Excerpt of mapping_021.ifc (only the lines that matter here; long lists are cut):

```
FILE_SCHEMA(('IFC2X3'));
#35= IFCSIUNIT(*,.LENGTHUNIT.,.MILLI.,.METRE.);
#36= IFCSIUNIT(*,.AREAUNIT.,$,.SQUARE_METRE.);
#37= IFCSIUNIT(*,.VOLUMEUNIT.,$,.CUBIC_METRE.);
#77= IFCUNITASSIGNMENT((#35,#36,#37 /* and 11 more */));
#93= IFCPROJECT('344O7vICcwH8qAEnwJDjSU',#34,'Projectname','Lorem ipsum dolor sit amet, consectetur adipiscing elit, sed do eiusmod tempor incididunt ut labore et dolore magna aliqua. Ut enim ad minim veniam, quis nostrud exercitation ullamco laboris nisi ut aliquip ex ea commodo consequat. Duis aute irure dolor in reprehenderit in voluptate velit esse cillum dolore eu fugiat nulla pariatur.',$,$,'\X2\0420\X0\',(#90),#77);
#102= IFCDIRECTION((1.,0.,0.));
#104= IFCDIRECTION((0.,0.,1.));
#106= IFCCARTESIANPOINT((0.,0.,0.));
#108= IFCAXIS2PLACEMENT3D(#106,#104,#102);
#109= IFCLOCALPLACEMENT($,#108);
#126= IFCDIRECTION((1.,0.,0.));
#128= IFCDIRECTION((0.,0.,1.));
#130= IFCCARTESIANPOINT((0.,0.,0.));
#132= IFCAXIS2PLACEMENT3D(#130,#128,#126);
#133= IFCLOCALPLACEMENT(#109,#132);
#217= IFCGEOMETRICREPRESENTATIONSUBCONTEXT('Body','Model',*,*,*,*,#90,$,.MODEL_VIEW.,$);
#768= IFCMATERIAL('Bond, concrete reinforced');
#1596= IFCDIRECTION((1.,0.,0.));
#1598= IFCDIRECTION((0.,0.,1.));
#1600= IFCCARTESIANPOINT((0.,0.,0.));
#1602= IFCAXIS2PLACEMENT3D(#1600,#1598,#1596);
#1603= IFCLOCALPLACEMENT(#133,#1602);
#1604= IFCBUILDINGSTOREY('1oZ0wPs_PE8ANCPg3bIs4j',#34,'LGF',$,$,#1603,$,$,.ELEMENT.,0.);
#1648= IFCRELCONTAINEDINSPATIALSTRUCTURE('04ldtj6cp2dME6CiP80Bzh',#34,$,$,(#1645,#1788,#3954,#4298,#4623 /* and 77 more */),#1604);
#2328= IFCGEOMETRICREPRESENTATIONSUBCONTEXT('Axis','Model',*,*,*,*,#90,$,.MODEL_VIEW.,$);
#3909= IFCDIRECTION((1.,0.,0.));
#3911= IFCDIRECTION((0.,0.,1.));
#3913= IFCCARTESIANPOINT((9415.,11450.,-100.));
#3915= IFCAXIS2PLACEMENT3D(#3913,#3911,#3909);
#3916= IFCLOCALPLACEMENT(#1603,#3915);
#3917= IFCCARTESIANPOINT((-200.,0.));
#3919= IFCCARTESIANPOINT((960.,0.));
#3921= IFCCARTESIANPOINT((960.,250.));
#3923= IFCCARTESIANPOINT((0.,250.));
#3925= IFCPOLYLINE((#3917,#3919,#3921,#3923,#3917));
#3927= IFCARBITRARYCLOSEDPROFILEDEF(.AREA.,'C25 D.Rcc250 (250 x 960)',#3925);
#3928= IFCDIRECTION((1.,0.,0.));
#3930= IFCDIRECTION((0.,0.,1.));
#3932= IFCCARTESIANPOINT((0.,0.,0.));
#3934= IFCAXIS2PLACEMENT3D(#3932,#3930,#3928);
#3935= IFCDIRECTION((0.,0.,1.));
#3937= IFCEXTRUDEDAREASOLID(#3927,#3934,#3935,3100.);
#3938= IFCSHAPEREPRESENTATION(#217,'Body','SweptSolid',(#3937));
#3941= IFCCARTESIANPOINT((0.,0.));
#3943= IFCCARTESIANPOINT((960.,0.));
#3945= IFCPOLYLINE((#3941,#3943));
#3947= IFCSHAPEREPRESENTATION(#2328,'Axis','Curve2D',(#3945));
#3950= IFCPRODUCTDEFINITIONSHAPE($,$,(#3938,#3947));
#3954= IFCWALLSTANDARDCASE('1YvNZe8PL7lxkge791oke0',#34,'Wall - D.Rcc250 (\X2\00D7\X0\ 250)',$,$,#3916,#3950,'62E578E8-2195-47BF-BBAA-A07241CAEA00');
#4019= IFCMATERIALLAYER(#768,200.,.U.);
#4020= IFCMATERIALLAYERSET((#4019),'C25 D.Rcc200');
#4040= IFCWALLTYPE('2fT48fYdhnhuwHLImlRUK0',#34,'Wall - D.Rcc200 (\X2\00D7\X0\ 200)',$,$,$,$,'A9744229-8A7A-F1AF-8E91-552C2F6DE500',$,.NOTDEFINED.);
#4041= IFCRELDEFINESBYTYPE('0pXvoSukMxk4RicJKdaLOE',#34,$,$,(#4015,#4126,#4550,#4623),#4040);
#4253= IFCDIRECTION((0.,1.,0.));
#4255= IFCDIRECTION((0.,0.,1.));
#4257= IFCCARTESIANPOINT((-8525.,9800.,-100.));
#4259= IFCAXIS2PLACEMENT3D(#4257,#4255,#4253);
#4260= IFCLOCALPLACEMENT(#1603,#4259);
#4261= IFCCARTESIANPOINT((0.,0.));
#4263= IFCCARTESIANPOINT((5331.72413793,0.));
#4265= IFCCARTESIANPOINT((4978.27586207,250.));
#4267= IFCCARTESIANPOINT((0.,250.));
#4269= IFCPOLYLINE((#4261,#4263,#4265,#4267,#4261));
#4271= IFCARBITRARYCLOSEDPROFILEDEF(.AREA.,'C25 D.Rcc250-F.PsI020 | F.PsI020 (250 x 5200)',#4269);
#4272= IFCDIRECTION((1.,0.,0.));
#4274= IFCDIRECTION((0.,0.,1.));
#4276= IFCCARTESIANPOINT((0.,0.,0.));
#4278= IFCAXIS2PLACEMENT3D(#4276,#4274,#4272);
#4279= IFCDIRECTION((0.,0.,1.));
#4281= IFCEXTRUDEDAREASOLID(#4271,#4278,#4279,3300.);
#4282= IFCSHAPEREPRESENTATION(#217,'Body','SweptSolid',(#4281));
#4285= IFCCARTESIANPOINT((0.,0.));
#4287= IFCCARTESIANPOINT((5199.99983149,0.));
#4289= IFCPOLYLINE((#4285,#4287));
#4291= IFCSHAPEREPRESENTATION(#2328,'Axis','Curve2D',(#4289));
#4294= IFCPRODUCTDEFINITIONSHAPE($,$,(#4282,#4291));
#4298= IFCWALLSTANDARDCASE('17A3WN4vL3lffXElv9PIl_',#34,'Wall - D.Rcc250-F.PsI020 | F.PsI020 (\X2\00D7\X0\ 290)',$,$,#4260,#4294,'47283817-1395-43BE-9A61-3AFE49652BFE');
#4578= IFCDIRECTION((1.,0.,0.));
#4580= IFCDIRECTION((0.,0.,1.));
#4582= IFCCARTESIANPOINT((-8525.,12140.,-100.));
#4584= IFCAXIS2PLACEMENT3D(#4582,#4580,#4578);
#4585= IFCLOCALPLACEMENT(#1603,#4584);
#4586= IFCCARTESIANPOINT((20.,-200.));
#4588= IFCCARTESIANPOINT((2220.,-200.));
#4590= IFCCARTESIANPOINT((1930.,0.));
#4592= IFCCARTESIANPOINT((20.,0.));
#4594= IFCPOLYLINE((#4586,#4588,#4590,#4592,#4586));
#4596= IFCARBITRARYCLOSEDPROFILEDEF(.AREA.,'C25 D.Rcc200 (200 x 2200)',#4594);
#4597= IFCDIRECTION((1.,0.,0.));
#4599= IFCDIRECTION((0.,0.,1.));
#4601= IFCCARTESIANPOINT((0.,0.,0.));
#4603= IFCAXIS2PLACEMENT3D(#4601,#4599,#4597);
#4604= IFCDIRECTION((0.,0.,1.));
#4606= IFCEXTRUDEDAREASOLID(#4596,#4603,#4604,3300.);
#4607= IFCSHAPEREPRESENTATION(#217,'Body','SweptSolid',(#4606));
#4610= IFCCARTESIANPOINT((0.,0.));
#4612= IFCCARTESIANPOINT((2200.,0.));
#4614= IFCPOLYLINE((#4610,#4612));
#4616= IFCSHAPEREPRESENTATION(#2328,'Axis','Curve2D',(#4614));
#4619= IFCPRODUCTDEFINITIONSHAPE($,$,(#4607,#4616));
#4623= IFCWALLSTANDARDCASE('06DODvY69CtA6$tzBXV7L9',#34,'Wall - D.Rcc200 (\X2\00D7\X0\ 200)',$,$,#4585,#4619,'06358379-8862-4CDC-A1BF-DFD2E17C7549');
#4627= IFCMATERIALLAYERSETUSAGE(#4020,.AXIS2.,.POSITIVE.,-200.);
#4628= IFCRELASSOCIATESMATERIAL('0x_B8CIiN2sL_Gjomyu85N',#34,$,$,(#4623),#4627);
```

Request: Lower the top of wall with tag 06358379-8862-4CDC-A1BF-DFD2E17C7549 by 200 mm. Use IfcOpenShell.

```python
import ifcopenshell
import ifcopenshell.geom
import ifcopenshell.util.representation
import ifcopenshell.util.shape
import ifcopenshell.util.unit

model = ifcopenshell.open("mapping_021.ifc")
unit_scale = ifcopenshell.util.unit.calculate_unit_scale(model)
settings = ifcopenshell.geom.settings()


def volume(element):
    """Net volume in cubic metres, openings subtracted."""
    shape = ifcopenshell.geom.create_shape(settings, element)
    return ifcopenshell.util.shape.get_volume(shape.geometry)


wall = model.by_guid("06DODvY69CtA6$tzBXV7L9")
before = volume(wall)

body = ifcopenshell.util.representation.get_representation(wall, "Model", "Body")
solid = body.Items[0]
old_height = solid.Depth
solid.Depth -= 0.2 / unit_scale
after = volume(wall)

print(f"height {old_height:g} -> {solid.Depth:g}, volume {before:.3f} -> {after:.3f} m3")

model.write("mapping_021_edited.ifc")
```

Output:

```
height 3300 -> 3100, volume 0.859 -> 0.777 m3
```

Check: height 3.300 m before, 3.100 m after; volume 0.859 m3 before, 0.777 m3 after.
